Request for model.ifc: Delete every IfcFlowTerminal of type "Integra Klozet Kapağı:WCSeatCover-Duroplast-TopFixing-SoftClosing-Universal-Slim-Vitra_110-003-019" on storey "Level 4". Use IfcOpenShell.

First a look at what the model holds.

```python
import ifcopenshell
import ifcopenshell.util.element

model = ifcopenshell.open("model.ifc")
print(model.schema)
storey = next(s for s in model.by_type("IfcBuildingStorey") if s.Name == "Level 4")
terminals = [e for e in ifcopenshell.util.element.get_decomposition(storey) if e.is_a("IfcFlowTerminal")]
seen = {}
for e in terminals:
    element_type = ifcopenshell.util.element.get_type(e)
    name = element_type.Name if element_type not in (None, e) else None
    seen[name] = seen.get(name, 0) + 1
for name, count in sorted(seen.items(), key=str):
    print(count, "x", name)
```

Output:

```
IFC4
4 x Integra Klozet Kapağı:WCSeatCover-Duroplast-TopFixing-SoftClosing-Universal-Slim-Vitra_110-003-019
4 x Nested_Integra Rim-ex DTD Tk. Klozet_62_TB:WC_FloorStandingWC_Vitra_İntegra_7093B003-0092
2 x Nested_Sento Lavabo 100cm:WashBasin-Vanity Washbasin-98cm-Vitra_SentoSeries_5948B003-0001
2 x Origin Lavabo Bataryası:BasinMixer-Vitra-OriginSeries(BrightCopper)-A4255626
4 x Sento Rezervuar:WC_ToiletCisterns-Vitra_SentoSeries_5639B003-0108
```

```python
import ifcopenshell
import ifcopenshell.api.root
import ifcopenshell.util.element

model = ifcopenshell.open("model.ifc")

storey = next(s for s in model.by_type("IfcBuildingStorey") if s.Name == "Level 4")
terminals = [e for e in ifcopenshell.util.element.get_decomposition(storey) if e.is_a("IfcFlowTerminal")]
targets = [e for e in terminals if (t := ifcopenshell.util.element.get_type(e)) not in (None, e) and t.Name == "Integra Klozet Kapağı:WCSeatCover-Duroplast-TopFixing-SoftClosing-Universal-Slim-Vitra_110-003-019"]

for e in targets:
    ifcopenshell.api.root.remove_product(model, product=e)
print(len(targets), "removed")

model.write("model_edited.ifc")
```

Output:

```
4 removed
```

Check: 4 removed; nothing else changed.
